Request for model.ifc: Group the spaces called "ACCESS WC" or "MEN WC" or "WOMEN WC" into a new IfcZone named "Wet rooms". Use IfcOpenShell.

First a look at what the model holds.

```python
import ifcopenshell

model = ifcopenshell.open("model.ifc")
print(model.schema)
seen = {}
for space in model.by_type("IfcSpace"):
    seen[space.LongName] = seen.get(space.LongName, 0) + 1
for name, count in sorted(seen.items(), key=str):
    print(count, "x", name)
print("zones:", [z.Name for z in model.by_type("IfcZone")][:20])
```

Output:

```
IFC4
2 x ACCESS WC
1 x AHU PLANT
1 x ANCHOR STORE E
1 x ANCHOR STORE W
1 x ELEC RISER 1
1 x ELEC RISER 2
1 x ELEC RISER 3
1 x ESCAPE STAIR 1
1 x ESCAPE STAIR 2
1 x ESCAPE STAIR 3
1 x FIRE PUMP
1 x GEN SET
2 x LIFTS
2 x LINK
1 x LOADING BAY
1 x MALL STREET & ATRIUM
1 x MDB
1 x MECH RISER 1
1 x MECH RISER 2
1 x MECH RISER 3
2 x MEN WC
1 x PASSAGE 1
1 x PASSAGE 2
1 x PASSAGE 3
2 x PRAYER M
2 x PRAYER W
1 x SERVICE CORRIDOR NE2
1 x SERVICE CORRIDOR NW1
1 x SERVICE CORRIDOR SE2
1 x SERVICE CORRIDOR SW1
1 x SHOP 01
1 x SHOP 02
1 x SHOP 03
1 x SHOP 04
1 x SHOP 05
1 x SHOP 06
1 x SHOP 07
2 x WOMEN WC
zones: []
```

```python
import ifcopenshell
import ifcopenshell.api.group
import ifcopenshell.api.root

model = ifcopenshell.open("model.ifc")

names = {"ACCESS WC", "MEN WC", "WOMEN WC"}
spaces = [s for s in model.by_type("IfcSpace") if s.LongName in names]

zone = ifcopenshell.api.root.create_entity(model, ifc_class="IfcZone", name="Wet rooms")
ifcopenshell.api.group.assign_group(model, products=spaces, group=zone)
print(len(spaces), "spaces in", zone.Name)

model.write("model_updated.ifc")
```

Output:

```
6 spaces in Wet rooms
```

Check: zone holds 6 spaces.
